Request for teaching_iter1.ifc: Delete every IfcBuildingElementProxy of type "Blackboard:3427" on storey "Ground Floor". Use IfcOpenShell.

First a look at what the model holds.

```python
import ifcopenshell
import ifcopenshell.util.element

model = ifcopenshell.open("teaching_iter1.ifc")
print(model.schema)
storey = next(s for s in model.by_type("IfcBuildingStorey") if s.Name == "Ground Floor")
proxies = [e for e in ifcopenshell.util.element.get_decomposition(storey) if e.is_a("IfcBuildingElementProxy")]
seen = {}
for e in proxies:
    element_type = ifcopenshell.util.element.get_type(e)
    name = element_type.Name if element_type not in (None, e) else None
    seen[name] = seen.get(name, 0) + 1
for name, count in sorted(seen.items(), key=str):
    print(count, "x", name)
```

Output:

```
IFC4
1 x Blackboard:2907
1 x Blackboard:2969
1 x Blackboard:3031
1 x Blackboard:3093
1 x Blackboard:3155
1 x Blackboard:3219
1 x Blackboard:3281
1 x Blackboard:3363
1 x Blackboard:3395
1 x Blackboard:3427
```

```python
import ifcopenshell
import ifcopenshell.api.root
import ifcopenshell.util.element

model = ifcopenshell.open("teaching_iter1.ifc")

storey = next(s for s in model.by_type("IfcBuildingStorey") if s.Name == "Ground Floor")
proxies = [e for e in ifcopenshell.util.element.get_decomposition(storey) if e.is_a("IfcBuildingElementProxy")]
targets = [e for e in proxies if (t := ifcopenshell.util.element.get_type(e)) not in (None, e) and t.Name == "Blackboard:3427"]

for e in targets:
    ifcopenshell.api.root.remove_product(model, product=e)
print(len(targets), "removed")

model.write("teaching_iter1_edited.ifc")
```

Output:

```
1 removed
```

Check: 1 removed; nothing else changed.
